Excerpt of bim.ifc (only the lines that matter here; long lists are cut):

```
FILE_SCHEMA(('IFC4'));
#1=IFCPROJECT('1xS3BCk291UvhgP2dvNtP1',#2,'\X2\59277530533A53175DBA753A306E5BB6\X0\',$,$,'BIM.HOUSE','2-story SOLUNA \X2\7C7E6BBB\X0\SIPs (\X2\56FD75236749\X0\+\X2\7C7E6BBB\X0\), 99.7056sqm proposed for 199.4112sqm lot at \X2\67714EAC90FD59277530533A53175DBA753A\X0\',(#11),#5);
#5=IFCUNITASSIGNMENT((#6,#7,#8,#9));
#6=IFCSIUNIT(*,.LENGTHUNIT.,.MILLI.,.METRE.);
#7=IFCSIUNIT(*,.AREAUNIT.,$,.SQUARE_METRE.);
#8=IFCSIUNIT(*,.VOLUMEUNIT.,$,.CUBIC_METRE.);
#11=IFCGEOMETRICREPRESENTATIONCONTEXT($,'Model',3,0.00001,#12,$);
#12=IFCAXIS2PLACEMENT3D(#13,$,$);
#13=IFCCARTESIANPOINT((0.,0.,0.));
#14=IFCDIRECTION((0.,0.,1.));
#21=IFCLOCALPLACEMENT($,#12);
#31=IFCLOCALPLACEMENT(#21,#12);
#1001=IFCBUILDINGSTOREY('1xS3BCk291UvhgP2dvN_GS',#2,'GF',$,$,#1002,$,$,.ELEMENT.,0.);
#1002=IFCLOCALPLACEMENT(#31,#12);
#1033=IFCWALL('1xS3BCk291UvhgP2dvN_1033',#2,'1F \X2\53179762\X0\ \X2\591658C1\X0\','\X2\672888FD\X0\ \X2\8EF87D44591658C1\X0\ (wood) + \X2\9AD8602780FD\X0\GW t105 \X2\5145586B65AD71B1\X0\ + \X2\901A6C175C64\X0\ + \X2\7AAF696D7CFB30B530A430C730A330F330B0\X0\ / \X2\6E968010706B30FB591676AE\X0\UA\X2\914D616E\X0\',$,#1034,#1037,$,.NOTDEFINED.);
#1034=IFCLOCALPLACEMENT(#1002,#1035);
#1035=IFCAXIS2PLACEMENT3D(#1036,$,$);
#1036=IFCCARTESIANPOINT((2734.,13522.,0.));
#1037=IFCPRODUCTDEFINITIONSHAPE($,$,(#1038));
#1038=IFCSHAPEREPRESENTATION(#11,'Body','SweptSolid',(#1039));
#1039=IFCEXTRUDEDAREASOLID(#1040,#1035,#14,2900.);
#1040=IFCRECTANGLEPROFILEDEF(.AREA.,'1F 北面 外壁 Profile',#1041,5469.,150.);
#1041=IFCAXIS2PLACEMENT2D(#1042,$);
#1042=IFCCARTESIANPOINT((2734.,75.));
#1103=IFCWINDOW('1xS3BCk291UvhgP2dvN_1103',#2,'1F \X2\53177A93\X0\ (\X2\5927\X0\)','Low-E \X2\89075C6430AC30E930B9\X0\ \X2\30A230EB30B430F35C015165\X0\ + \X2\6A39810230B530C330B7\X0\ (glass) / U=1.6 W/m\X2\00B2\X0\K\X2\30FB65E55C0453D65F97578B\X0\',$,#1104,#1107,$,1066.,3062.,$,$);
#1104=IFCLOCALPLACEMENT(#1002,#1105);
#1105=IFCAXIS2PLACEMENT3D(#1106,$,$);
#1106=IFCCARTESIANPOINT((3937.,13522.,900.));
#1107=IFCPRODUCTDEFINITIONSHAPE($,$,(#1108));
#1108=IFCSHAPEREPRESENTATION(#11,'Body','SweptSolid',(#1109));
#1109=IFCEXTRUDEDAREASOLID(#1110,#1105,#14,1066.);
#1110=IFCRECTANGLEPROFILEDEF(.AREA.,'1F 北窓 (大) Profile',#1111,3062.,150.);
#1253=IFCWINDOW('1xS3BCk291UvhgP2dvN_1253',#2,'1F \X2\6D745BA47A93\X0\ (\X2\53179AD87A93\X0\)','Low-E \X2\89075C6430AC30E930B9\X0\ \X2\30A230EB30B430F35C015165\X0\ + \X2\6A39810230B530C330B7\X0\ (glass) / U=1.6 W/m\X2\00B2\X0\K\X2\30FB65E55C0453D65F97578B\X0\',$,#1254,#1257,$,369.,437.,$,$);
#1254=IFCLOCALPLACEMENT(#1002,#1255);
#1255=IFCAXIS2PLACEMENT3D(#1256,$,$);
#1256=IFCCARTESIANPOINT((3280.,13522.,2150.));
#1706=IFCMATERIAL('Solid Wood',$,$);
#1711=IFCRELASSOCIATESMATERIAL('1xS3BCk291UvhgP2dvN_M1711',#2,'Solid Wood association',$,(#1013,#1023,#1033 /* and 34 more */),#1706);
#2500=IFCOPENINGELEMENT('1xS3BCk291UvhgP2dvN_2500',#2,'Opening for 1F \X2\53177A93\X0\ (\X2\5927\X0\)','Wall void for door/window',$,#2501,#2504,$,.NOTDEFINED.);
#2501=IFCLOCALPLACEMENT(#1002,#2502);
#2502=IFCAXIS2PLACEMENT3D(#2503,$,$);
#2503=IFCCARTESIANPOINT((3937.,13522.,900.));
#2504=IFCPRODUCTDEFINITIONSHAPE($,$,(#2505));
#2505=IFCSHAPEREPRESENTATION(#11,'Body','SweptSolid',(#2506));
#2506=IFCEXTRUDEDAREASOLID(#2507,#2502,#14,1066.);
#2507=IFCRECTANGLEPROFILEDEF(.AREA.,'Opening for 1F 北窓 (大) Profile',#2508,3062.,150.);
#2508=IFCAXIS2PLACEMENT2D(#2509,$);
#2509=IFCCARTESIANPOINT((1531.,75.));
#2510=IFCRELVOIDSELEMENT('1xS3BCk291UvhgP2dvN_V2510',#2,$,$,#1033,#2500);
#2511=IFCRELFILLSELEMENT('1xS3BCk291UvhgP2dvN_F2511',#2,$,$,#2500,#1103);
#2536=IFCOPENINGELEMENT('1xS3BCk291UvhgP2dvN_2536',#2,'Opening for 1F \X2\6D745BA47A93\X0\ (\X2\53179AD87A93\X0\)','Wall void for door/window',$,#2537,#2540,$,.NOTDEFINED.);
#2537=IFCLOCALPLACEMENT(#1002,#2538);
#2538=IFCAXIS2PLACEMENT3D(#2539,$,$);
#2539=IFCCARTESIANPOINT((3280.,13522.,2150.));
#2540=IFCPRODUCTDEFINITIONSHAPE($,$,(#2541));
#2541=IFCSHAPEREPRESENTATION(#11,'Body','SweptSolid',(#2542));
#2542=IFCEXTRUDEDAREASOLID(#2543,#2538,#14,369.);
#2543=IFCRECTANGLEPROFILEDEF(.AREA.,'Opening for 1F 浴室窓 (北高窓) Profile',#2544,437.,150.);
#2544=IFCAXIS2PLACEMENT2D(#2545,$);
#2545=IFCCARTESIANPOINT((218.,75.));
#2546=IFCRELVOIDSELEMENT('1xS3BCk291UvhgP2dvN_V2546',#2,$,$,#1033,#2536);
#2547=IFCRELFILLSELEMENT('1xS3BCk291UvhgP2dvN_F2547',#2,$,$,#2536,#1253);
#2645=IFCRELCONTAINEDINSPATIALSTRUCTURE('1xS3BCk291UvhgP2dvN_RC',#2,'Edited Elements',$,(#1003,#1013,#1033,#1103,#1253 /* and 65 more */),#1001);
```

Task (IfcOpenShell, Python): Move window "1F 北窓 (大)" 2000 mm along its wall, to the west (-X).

```python
import ifcopenshell
import ifcopenshell.api.geometry
import ifcopenshell.util.placement

model = ifcopenshell.open("bim.ifc")

window = model.by_guid("1xS3BCk291UvhgP2dvN_1103")
opening = window.FillsVoids[0].RelatingOpeningElement
wall = opening.VoidsElements[0].RelatingBuildingElement

wall_matrix = ifcopenshell.util.placement.get_local_placement(wall.ObjectPlacement)
shift = wall_matrix[:3, 0] * -2000.0
before = ifcopenshell.util.placement.get_local_placement(window.ObjectPlacement)[:3, 3].copy()

# The window is not placed relative to its opening, so move both.
for product in (opening, window):
    matrix = ifcopenshell.util.placement.get_local_placement(product.ObjectPlacement)
    matrix[:3, 3] += shift
    ifcopenshell.api.geometry.edit_object_placement(model, product=product, matrix=matrix, is_si=False)

after = ifcopenshell.util.placement.get_local_placement(window.ObjectPlacement)[:3, 3]
print("window moved by", (after - before).round(3) + 0.0)

model.write("bim-out.ifc")
```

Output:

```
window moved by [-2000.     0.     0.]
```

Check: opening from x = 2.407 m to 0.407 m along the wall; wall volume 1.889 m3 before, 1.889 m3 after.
